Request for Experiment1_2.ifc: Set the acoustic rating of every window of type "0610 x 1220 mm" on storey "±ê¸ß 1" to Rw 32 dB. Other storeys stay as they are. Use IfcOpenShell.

First a look at what the model holds.

```python
import ifcopenshell
import ifcopenshell.util.element

model = ifcopenshell.open("Experiment1_2.ifc")
print(model.schema)
storey = next(s for s in model.by_type("IfcBuildingStorey") if s.Name == "±ê¸ß 1")
windows = [e for e in ifcopenshell.util.element.get_decomposition(storey) if e.is_a("IfcWindow")]
seen = {}
for e in windows:
    element_type = ifcopenshell.util.element.get_type(e)
    key = (element_type.Name if element_type != e and element_type else None, ifcopenshell.util.element.get_pset(e, "Pset_WindowCommon", "AcousticRating"))
    seen[key] = seen.get(key, 0) + 1
for (name, value), count in sorted(seen.items(), key=str):
    print(count, "x", name, "|", value)
```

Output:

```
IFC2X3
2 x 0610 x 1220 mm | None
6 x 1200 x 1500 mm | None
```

```python
import ifcopenshell
import ifcopenshell.api.pset
import ifcopenshell.util.element

model = ifcopenshell.open("Experiment1_2.ifc")

storey = next(s for s in model.by_type("IfcBuildingStorey") if s.Name == "±ê¸ß 1")
windows = [e for e in ifcopenshell.util.element.get_decomposition(storey) if e.is_a("IfcWindow")]

count = 0
for e in windows:
    element_type = ifcopenshell.util.element.get_type(e)
    if element_type in (None, e) or element_type.Name != "0610 x 1220 mm":
        continue
    # add_pset returns the element's existing set when there is one.
    pset = ifcopenshell.api.pset.add_pset(model, product=e, name="Pset_WindowCommon")
    ifcopenshell.api.pset.edit_pset(model, pset=pset, properties={"AcousticRating": "Rw 32 dB"})
    count += 1

print(count, "windows updated")

model.write("Experiment1_2_rev.ifc")
```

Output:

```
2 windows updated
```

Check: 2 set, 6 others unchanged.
